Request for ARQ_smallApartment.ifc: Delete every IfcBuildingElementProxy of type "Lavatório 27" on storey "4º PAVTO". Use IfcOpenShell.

First a look at what the model holds.

```python
import ifcopenshell
import ifcopenshell.util.element

model = ifcopenshell.open("ARQ_smallApartment.ifc")
print(model.schema)
storey = next(s for s in model.by_type("IfcBuildingStorey") if s.Name == "4º PAVTO")
proxies = [e for e in ifcopenshell.util.element.get_decomposition(storey) if e.is_a("IfcBuildingElementProxy")]
seen = {}
for e in proxies:
    element_type = ifcopenshell.util.element.get_type(e)
    name = element_type.Name if element_type not in (None, e) else None
    seen[name] = seen.get(name, 0) + 1
for name, count in sorted(seen.items(), key=str):
    print(count, "x", name)
```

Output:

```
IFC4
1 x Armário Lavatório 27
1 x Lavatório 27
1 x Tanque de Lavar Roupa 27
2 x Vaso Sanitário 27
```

```python
import ifcopenshell
import ifcopenshell.api.root
import ifcopenshell.util.element

model = ifcopenshell.open("ARQ_smallApartment.ifc")

storey = next(s for s in model.by_type("IfcBuildingStorey") if s.Name == "4º PAVTO")
proxies = [e for e in ifcopenshell.util.element.get_decomposition(storey) if e.is_a("IfcBuildingElementProxy")]
targets = [e for e in proxies if (t := ifcopenshell.util.element.get_type(e)) not in (None, e) and t.Name == "Lavatório 27"]

for e in targets:
    ifcopenshell.api.root.remove_product(model, product=e)
print(len(targets), "removed")

model.write("ARQ_smallApartment-out.ifc")
```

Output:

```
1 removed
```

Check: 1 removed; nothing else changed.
